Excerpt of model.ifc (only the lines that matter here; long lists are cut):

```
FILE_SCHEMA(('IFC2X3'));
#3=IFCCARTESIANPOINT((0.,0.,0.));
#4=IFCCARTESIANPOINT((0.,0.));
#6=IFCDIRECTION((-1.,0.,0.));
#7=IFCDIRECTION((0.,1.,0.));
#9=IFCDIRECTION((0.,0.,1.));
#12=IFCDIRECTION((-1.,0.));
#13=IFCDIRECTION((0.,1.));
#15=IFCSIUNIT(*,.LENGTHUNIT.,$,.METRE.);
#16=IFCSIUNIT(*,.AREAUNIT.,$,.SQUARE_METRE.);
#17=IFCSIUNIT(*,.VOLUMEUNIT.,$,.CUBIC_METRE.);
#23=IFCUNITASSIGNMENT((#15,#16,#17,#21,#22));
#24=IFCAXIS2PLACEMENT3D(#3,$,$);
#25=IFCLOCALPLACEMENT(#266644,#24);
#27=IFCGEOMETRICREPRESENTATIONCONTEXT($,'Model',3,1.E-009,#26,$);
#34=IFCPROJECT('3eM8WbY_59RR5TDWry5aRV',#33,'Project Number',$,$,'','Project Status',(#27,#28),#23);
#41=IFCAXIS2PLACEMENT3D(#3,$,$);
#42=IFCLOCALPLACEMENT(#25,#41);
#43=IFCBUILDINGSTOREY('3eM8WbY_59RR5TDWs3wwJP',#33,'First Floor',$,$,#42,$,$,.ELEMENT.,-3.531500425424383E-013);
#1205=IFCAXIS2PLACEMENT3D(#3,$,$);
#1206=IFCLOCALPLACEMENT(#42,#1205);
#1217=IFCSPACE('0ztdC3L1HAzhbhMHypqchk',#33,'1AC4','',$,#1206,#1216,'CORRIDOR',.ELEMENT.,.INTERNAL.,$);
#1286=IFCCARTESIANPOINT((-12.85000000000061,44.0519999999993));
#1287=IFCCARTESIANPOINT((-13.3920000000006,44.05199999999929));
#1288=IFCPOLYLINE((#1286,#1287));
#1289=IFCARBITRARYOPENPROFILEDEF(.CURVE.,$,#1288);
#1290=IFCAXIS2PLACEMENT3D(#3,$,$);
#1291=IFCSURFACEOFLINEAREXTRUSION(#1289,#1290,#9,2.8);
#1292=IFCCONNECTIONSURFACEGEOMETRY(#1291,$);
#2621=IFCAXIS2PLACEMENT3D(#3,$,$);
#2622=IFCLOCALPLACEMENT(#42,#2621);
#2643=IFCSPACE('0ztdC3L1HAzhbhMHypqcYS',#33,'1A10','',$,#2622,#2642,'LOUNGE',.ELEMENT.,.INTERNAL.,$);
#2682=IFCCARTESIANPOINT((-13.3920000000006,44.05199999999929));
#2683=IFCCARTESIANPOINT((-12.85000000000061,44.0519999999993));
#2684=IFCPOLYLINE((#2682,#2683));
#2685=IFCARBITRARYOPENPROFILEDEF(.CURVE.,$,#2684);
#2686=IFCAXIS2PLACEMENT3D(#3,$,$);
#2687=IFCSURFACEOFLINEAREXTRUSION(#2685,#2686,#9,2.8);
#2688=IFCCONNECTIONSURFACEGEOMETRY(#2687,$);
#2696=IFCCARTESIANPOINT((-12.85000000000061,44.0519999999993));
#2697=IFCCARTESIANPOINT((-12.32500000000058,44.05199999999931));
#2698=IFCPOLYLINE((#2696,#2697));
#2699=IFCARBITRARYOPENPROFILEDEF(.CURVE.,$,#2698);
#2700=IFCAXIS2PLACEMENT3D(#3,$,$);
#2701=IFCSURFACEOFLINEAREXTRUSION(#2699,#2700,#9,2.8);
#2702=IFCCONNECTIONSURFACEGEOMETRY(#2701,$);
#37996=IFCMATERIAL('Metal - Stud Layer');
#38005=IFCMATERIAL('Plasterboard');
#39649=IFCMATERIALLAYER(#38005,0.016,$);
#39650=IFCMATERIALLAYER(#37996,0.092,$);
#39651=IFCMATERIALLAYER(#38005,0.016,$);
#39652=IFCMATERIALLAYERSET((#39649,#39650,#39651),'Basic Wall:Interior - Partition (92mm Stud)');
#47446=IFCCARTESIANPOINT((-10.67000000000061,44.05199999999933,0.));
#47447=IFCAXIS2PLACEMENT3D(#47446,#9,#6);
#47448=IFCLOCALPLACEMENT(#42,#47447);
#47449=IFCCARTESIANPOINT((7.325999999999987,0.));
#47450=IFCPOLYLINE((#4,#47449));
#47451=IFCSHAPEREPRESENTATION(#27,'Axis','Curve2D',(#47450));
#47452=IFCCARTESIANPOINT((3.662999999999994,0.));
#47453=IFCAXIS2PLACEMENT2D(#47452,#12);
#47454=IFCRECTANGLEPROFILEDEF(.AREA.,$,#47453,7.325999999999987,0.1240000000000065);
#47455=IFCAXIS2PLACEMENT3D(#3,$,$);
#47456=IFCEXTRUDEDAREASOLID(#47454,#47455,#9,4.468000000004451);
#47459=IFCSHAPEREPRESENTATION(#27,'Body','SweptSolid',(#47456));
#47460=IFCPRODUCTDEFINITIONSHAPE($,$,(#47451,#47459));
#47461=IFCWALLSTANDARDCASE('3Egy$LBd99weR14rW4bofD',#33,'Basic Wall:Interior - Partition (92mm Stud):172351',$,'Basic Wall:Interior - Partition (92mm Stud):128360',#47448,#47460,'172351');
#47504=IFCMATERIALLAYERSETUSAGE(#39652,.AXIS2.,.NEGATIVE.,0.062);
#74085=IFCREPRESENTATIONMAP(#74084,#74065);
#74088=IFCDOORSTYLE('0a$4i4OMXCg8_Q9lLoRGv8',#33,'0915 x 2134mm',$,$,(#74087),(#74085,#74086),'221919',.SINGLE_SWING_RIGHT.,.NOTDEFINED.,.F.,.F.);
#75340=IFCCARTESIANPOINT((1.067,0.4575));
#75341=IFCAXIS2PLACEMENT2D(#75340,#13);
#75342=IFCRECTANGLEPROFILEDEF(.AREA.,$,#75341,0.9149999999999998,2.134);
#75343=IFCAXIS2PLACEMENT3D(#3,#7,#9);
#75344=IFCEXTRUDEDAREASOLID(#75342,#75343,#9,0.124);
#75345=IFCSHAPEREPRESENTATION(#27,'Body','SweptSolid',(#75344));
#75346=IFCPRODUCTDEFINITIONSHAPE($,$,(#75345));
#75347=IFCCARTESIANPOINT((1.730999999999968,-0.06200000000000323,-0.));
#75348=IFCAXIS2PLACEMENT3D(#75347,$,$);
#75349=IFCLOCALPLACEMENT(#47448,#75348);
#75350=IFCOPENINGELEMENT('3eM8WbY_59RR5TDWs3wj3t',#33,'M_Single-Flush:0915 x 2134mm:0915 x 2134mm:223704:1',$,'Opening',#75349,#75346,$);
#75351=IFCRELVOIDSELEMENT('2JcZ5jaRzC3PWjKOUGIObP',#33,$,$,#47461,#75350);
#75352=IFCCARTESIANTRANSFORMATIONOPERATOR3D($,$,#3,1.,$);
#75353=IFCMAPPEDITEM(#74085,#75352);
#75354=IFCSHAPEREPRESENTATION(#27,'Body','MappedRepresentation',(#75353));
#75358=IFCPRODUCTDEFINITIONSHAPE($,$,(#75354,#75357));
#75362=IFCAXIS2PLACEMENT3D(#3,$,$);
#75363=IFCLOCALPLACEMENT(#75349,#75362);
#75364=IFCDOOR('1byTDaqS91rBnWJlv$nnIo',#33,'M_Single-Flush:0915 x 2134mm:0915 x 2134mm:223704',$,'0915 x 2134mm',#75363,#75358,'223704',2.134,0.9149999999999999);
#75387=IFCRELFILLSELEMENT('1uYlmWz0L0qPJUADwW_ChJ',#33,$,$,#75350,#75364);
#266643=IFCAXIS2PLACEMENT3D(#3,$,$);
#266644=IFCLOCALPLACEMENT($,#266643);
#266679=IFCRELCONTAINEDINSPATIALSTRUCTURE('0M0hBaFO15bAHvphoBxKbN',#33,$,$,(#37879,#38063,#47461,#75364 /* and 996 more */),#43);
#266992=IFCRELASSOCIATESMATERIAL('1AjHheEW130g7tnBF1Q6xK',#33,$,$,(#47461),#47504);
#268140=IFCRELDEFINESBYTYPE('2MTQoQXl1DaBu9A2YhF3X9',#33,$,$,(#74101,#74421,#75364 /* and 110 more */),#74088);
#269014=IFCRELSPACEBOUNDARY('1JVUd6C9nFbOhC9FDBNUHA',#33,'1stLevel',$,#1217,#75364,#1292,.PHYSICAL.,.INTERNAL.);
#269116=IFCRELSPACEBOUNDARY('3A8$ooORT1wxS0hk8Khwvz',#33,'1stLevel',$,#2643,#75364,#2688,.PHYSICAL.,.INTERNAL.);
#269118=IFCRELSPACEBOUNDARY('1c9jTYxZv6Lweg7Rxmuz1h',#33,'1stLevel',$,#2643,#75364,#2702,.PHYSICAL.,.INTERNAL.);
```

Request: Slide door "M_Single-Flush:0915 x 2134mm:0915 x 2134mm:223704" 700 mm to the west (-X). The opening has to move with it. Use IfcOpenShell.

```python
import numpy as np
import ifcopenshell
import ifcopenshell.api.geometry
import ifcopenshell.util.placement
import ifcopenshell.util.unit

model = ifcopenshell.open("model.ifc")
unit_scale = ifcopenshell.util.unit.calculate_unit_scale(model)

door = model.by_guid("1byTDaqS91rBnWJlv$nnIo")
opening = door.FillsVoids[0].RelatingOpeningElement
wall = opening.VoidsElements[0].RelatingBuildingElement

wall_matrix = ifcopenshell.util.placement.get_local_placement(wall.ObjectPlacement)
shift = wall_matrix[:3, 0] * 0.7 / unit_scale
before = ifcopenshell.util.placement.get_local_placement(door.ObjectPlacement)[:3, 3].copy()

# The door is placed relative to its opening, so it follows when the opening moves.
matrix = ifcopenshell.util.placement.get_local_placement(opening.ObjectPlacement)
matrix[:3, 3] += shift
ifcopenshell.api.geometry.edit_object_placement(
    model, product=opening, matrix=matrix, is_si=False, should_transform_children=True
)

# Space boundary surfaces are stored in each space's coordinates; move them too.
for rel in door.ProvidesBoundaries:
    if not rel.ConnectionGeometry:
        continue
    surface = rel.ConnectionGeometry.SurfaceOnRelatingElement
    space_matrix = ifcopenshell.util.placement.get_local_placement(rel.RelatingSpace.ObjectPlacement)
    point = np.array(surface.Position.Location.Coordinates) + space_matrix[:3, :3].T @ shift
    surface.Position = model.createIfcAxis2Placement3D(
        model.createIfcCartesianPoint(point.tolist()), surface.Position.Axis, surface.Position.RefDirection
    )

after = ifcopenshell.util.placement.get_local_placement(door.ObjectPlacement)[:3, 3]
print("door moved by", (after - before).round(3) + 0.0)

model.write("model-out.ifc")
```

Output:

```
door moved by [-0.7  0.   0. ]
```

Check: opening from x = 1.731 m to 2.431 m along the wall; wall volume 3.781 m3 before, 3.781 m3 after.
